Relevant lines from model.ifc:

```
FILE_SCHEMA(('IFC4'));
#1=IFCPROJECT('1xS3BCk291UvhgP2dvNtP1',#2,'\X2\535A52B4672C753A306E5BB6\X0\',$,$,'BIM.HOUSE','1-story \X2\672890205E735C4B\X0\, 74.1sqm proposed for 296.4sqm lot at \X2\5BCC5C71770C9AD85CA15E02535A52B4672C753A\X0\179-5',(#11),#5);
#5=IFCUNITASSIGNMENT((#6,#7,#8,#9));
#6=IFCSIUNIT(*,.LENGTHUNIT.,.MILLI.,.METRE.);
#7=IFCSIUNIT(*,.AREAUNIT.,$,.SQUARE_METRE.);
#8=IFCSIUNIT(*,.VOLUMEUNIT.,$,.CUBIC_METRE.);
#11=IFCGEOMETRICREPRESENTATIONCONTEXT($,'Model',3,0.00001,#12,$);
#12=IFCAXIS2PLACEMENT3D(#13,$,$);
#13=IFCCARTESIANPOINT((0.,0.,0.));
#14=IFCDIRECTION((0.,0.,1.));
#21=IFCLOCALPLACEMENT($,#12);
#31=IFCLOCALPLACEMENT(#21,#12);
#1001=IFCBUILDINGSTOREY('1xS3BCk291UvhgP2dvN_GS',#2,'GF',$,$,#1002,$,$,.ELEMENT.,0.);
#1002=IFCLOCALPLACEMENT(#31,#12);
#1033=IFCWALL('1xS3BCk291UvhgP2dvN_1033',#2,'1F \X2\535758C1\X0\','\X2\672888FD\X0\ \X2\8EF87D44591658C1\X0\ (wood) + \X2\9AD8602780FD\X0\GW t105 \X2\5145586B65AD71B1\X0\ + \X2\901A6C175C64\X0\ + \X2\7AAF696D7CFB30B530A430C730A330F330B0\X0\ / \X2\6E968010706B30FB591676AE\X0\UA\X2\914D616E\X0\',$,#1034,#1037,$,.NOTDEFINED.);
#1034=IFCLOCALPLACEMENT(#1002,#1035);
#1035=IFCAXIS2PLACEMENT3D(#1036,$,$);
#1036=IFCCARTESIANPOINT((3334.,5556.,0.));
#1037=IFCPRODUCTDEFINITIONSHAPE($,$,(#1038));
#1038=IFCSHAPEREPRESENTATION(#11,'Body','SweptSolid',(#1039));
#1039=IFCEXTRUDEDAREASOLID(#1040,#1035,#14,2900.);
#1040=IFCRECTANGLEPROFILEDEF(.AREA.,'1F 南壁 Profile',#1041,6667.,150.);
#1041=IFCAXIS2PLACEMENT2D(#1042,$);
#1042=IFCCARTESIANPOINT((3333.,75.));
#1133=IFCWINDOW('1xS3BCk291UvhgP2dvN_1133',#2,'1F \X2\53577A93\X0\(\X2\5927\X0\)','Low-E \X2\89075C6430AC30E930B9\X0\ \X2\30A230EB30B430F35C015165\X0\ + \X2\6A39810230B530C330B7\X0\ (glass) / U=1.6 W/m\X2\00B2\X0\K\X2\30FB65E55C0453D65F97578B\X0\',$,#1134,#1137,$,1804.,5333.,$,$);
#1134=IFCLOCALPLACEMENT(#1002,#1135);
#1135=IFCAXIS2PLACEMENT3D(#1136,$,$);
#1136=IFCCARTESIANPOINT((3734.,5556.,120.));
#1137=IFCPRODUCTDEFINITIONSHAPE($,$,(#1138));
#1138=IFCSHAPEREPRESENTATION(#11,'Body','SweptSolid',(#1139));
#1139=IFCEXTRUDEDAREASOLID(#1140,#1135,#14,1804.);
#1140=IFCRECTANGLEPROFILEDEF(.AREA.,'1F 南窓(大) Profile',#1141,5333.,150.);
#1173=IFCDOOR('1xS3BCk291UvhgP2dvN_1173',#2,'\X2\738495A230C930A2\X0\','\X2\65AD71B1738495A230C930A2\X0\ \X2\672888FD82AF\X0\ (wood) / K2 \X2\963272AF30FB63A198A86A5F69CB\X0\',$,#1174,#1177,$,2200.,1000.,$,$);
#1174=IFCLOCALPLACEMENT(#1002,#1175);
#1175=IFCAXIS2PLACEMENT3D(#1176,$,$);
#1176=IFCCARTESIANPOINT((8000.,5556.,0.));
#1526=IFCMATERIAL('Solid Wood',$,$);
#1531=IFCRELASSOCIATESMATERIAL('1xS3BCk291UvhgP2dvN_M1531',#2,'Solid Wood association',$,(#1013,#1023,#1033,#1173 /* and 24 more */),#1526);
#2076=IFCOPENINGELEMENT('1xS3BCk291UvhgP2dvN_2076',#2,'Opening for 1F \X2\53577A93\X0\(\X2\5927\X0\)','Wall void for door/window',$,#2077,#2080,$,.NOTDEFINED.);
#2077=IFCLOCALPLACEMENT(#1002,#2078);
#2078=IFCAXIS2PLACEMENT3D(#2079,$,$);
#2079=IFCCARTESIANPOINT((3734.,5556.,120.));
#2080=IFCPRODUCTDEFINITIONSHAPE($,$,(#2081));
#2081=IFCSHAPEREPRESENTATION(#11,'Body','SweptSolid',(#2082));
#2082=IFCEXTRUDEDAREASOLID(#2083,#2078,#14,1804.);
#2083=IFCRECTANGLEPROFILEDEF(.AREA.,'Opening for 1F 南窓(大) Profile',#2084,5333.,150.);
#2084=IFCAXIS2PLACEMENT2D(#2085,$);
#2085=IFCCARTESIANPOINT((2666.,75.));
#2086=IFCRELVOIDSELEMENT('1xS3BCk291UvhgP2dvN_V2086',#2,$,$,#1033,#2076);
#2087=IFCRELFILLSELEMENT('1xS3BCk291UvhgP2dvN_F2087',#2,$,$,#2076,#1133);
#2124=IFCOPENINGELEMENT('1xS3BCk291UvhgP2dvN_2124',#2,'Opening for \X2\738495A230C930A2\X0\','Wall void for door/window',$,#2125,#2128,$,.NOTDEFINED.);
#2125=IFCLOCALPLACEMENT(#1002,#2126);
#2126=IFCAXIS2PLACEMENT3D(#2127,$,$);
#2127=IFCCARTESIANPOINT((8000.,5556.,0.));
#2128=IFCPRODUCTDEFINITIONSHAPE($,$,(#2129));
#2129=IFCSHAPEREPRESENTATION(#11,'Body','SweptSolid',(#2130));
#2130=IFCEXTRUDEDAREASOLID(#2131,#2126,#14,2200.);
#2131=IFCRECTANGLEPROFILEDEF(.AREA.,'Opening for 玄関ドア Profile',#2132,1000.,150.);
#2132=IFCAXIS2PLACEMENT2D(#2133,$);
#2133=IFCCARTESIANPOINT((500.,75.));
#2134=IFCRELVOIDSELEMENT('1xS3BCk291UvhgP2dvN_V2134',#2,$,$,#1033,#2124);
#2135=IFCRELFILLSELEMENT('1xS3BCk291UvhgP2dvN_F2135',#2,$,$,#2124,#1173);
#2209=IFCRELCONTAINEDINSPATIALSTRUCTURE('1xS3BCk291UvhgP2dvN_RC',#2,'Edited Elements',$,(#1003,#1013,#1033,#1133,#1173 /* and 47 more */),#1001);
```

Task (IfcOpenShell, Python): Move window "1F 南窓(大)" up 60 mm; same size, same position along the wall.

```python
import numpy as np
import ifcopenshell
import ifcopenshell.api.geometry
import ifcopenshell.util.placement
import ifcopenshell.util.unit

model = ifcopenshell.open("model.ifc")
unit_scale = ifcopenshell.util.unit.calculate_unit_scale(model)

window = model.by_guid("1xS3BCk291UvhgP2dvN_1133")
opening = window.FillsVoids[0].RelatingOpeningElement
dz = 0.06 / unit_scale

shift = np.array([0.0, 0.0, dz])
# The window is not placed relative to its opening, so move both.
for product in (opening, window):
    matrix = ifcopenshell.util.placement.get_local_placement(product.ObjectPlacement)
    matrix[:3, 3] += shift
    ifcopenshell.api.geometry.edit_object_placement(model, product=product, matrix=matrix, is_si=False)

print(f"moved by {dz * unit_scale:+.3f} m")

model.write("model_updated.ifc")
```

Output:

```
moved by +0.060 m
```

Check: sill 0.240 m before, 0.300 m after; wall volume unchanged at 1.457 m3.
